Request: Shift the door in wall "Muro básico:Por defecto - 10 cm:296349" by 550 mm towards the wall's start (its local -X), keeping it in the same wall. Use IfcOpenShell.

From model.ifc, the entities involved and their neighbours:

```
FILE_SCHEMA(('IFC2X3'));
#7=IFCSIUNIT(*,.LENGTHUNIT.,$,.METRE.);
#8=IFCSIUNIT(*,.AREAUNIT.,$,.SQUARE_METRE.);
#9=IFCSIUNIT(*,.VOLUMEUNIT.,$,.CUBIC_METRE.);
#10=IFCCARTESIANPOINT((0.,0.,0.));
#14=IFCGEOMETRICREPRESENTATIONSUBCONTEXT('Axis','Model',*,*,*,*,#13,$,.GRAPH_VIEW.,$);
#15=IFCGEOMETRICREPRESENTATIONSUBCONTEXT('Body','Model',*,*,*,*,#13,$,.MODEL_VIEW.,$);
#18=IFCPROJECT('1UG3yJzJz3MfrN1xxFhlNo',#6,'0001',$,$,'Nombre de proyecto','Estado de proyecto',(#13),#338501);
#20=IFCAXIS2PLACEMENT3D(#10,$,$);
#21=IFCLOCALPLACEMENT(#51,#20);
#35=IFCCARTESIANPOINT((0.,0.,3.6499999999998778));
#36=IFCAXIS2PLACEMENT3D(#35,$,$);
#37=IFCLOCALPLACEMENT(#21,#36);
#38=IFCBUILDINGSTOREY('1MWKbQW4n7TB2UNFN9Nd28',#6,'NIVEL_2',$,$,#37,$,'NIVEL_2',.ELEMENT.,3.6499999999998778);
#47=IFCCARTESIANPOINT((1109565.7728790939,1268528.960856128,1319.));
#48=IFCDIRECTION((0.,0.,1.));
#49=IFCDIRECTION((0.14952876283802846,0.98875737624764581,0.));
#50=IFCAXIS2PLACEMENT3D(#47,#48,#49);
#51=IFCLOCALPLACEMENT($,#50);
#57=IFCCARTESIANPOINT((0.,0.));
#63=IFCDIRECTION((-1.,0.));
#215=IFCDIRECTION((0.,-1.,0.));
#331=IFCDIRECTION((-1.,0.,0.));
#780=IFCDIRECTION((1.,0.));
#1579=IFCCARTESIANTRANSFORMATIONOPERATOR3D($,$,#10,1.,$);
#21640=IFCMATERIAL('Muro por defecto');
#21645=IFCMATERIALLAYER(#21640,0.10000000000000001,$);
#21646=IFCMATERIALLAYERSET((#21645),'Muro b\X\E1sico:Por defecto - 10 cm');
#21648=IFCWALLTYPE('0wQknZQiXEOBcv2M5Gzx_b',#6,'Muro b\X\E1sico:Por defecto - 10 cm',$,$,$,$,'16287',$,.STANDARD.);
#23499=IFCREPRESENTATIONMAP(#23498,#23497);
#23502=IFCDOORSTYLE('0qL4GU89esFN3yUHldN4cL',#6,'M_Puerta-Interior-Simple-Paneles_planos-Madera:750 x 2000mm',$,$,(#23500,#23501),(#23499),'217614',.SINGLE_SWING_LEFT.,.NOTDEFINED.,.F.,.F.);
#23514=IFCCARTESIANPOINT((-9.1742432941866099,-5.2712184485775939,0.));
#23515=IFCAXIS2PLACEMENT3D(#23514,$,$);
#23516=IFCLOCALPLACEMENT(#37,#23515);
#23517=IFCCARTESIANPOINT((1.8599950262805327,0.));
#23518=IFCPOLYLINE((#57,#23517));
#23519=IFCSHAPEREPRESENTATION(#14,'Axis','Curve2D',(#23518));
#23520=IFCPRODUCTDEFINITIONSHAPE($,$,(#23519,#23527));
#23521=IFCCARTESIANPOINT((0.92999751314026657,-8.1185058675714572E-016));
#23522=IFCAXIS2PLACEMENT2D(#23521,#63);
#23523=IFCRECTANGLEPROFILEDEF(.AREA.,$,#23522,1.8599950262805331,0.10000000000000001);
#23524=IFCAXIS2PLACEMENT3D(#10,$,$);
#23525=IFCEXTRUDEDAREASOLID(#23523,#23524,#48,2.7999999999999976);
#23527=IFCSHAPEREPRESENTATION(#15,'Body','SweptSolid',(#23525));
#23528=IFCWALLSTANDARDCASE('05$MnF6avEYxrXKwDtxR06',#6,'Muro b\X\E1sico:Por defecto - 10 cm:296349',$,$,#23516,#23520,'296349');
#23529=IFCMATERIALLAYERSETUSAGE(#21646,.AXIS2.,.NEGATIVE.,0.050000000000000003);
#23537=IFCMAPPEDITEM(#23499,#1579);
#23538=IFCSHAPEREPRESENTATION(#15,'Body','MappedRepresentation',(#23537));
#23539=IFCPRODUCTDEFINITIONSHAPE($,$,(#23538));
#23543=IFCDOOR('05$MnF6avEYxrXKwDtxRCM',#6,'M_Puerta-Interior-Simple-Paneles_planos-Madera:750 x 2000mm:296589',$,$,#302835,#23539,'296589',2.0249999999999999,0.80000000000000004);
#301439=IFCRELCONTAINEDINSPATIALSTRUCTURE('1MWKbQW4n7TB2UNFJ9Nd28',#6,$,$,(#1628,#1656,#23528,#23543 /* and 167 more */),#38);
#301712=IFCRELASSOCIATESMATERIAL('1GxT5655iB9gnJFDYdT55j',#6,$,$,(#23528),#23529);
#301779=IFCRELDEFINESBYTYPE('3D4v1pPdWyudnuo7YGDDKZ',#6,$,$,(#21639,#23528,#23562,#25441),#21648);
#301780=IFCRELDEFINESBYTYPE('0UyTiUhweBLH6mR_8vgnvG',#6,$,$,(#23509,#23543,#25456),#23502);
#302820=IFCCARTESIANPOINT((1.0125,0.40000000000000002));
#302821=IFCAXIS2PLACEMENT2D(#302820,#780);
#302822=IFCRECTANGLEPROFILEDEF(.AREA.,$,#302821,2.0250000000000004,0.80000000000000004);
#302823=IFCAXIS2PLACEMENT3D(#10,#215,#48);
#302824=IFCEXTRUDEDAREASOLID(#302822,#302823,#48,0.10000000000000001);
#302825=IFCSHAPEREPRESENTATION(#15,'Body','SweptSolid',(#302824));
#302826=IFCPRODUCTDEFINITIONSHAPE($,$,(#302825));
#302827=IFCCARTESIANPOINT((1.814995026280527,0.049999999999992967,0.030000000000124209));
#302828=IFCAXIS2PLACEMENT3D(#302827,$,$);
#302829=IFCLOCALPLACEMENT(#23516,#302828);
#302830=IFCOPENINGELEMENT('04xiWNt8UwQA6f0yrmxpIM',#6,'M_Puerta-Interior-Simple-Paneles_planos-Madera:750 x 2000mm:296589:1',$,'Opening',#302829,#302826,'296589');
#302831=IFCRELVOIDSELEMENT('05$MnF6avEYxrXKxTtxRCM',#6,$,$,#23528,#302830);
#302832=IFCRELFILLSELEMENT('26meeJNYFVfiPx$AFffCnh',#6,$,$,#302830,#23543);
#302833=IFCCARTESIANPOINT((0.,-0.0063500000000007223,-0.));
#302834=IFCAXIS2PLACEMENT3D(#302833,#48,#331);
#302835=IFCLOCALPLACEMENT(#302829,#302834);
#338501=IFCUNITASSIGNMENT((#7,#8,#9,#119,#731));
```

```python
import ifcopenshell
import ifcopenshell.api.geometry
import ifcopenshell.util.placement

model = ifcopenshell.open("model.ifc")

door = model.by_id(23543)
opening = door.FillsVoids[0].RelatingOpeningElement
wall = opening.VoidsElements[0].RelatingBuildingElement

wall_matrix = ifcopenshell.util.placement.get_local_placement(wall.ObjectPlacement)
shift = wall_matrix[:3, 0] * -0.55
before = ifcopenshell.util.placement.get_local_placement(door.ObjectPlacement)[:3, 3].copy()

# The door is placed relative to its opening, so it follows when the opening moves.
matrix = ifcopenshell.util.placement.get_local_placement(opening.ObjectPlacement)
matrix[:3, 3] += shift
ifcopenshell.api.geometry.edit_object_placement(
    model, product=opening, matrix=matrix, is_si=False, should_transform_children=True
)

after = ifcopenshell.util.placement.get_local_placement(door.ObjectPlacement)[:3, 3]
print("door moved by", (after - before).round(3) + 0.0)

model.write("model_edited.ifc")
```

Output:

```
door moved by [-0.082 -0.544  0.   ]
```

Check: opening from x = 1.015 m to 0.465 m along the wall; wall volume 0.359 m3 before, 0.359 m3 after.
